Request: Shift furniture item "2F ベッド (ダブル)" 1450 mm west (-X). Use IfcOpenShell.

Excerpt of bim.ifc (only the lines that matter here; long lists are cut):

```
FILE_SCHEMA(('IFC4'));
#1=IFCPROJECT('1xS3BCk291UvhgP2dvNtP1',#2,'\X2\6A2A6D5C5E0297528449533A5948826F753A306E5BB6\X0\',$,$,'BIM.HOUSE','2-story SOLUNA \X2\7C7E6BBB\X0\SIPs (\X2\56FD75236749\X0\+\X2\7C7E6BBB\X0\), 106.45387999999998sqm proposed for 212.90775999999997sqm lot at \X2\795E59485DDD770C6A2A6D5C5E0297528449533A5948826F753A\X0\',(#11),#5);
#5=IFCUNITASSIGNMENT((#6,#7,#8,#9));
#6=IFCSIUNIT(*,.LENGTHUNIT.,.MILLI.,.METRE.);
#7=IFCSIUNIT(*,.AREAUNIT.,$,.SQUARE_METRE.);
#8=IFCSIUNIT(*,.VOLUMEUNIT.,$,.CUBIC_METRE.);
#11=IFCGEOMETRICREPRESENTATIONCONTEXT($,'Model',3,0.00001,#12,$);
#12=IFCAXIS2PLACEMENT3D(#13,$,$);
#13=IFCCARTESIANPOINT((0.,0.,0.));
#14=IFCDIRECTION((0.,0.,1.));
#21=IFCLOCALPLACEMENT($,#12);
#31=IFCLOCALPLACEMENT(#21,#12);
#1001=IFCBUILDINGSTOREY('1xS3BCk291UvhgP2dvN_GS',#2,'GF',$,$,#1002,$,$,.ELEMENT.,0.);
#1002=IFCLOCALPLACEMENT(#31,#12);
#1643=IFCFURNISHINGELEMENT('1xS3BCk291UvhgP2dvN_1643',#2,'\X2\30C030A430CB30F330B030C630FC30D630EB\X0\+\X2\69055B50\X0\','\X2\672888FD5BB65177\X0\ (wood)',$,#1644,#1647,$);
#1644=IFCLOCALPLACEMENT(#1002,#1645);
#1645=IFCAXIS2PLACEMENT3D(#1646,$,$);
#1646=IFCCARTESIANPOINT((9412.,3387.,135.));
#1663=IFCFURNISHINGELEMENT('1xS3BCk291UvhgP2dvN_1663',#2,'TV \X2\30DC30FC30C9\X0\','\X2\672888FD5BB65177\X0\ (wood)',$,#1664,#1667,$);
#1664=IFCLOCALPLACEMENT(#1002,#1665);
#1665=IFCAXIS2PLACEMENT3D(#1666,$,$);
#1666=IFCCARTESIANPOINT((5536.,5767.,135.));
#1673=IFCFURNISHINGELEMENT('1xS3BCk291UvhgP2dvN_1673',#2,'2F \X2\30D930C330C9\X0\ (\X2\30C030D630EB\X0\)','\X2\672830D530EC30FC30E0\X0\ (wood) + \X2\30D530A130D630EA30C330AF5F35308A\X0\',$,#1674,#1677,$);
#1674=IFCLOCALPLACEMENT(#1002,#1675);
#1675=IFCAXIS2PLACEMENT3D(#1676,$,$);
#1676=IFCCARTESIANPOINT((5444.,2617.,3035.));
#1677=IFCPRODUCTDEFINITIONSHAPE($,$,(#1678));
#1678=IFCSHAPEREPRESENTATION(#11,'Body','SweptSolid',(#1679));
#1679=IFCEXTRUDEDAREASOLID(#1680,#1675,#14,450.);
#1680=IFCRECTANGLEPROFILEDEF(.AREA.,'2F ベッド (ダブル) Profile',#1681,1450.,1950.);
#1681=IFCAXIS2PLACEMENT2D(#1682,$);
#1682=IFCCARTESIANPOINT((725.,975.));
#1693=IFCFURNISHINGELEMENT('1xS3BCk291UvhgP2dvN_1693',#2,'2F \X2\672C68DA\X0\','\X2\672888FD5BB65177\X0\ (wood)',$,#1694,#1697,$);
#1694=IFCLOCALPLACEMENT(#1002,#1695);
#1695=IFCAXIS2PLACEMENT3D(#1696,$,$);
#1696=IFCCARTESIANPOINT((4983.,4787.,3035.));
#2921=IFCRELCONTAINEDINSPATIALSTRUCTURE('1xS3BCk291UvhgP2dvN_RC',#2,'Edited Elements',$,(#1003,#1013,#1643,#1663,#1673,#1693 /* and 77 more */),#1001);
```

```python
import ifcopenshell
import ifcopenshell.api.geometry
import ifcopenshell.util.placement

model = ifcopenshell.open("bim.ifc")

item = model.by_id(1673)
matrix = ifcopenshell.util.placement.get_local_placement(item.ObjectPlacement)
matrix[0, 3] -= 1450.0
ifcopenshell.api.geometry.edit_object_placement(model, product=item, matrix=matrix, is_si=False)

print(ifcopenshell.util.placement.get_local_placement(item.ObjectPlacement).round(3) + 0.0)

model.write("bim_edited.ifc")
```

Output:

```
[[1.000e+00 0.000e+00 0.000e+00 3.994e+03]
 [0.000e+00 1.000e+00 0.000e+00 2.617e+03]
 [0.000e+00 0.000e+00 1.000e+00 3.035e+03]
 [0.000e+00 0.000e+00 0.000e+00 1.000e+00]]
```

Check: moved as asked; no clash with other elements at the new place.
